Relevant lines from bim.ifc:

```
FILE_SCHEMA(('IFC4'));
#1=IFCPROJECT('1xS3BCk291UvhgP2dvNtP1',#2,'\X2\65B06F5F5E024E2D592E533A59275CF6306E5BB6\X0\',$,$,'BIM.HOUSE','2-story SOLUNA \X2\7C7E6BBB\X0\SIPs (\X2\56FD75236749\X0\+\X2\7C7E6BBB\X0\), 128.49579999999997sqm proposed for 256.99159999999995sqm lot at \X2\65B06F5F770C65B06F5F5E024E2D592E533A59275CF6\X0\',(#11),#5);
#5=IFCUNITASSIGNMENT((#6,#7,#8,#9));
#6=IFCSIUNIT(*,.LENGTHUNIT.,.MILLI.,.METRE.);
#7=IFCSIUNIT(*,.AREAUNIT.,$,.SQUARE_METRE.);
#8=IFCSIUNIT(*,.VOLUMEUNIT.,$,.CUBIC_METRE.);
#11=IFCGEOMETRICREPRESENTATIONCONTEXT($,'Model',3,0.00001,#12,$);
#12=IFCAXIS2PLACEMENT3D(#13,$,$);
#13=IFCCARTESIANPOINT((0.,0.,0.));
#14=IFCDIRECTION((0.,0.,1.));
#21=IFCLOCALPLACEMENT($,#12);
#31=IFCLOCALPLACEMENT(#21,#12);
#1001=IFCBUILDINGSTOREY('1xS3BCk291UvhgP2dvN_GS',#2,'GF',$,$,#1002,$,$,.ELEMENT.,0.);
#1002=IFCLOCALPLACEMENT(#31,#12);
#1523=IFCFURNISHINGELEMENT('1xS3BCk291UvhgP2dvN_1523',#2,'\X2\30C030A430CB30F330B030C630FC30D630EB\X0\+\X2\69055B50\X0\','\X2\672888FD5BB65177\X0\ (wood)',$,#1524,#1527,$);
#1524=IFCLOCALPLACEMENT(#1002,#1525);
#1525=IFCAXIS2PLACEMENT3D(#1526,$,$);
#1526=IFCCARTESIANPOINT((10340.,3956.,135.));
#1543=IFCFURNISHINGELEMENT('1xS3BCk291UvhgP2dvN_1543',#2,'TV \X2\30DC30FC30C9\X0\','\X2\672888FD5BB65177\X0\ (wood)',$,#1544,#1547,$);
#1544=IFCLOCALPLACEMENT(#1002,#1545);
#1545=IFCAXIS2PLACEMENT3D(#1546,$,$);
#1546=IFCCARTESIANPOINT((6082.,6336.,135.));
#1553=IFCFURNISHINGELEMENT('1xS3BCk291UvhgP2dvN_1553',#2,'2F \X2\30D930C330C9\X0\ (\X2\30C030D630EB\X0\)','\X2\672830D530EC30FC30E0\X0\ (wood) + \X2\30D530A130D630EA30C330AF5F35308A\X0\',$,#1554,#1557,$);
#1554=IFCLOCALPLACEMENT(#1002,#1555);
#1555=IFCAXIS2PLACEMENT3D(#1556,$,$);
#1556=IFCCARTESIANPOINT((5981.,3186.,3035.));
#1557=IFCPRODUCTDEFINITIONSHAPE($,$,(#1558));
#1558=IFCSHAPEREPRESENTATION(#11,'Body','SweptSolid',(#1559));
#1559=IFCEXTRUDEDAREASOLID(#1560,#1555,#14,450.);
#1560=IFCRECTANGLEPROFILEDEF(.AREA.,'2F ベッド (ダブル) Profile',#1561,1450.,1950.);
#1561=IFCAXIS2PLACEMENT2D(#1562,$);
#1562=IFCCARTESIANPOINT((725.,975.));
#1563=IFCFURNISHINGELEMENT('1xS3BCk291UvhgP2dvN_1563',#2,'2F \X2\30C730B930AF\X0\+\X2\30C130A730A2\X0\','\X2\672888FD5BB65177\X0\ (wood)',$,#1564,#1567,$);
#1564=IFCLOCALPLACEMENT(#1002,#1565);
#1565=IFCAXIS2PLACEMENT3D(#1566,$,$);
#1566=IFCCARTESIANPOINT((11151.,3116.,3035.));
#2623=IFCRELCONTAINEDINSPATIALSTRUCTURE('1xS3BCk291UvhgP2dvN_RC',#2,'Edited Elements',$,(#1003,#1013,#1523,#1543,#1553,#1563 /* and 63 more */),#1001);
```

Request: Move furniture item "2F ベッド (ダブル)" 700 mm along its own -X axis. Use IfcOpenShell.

```python
import ifcopenshell
import ifcopenshell.api.geometry
import ifcopenshell.util.placement
import ifcopenshell.util.unit

model = ifcopenshell.open("bim.ifc")
unit_scale = ifcopenshell.util.unit.calculate_unit_scale(model)

item = model.by_guid("1xS3BCk291UvhgP2dvN_1553")
matrix = ifcopenshell.util.placement.get_local_placement(item.ObjectPlacement)
matrix[:3, 3] -= matrix[:3, 0] * 0.7 / unit_scale
ifcopenshell.api.geometry.edit_object_placement(model, product=item, matrix=matrix, is_si=False)

print(ifcopenshell.util.placement.get_local_placement(item.ObjectPlacement).round(3) + 0.0)

model.write("bim_edited.ifc")
```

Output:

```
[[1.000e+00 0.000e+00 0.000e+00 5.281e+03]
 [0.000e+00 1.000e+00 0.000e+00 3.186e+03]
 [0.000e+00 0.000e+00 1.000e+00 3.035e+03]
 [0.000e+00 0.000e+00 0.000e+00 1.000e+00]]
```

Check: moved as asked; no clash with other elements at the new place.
